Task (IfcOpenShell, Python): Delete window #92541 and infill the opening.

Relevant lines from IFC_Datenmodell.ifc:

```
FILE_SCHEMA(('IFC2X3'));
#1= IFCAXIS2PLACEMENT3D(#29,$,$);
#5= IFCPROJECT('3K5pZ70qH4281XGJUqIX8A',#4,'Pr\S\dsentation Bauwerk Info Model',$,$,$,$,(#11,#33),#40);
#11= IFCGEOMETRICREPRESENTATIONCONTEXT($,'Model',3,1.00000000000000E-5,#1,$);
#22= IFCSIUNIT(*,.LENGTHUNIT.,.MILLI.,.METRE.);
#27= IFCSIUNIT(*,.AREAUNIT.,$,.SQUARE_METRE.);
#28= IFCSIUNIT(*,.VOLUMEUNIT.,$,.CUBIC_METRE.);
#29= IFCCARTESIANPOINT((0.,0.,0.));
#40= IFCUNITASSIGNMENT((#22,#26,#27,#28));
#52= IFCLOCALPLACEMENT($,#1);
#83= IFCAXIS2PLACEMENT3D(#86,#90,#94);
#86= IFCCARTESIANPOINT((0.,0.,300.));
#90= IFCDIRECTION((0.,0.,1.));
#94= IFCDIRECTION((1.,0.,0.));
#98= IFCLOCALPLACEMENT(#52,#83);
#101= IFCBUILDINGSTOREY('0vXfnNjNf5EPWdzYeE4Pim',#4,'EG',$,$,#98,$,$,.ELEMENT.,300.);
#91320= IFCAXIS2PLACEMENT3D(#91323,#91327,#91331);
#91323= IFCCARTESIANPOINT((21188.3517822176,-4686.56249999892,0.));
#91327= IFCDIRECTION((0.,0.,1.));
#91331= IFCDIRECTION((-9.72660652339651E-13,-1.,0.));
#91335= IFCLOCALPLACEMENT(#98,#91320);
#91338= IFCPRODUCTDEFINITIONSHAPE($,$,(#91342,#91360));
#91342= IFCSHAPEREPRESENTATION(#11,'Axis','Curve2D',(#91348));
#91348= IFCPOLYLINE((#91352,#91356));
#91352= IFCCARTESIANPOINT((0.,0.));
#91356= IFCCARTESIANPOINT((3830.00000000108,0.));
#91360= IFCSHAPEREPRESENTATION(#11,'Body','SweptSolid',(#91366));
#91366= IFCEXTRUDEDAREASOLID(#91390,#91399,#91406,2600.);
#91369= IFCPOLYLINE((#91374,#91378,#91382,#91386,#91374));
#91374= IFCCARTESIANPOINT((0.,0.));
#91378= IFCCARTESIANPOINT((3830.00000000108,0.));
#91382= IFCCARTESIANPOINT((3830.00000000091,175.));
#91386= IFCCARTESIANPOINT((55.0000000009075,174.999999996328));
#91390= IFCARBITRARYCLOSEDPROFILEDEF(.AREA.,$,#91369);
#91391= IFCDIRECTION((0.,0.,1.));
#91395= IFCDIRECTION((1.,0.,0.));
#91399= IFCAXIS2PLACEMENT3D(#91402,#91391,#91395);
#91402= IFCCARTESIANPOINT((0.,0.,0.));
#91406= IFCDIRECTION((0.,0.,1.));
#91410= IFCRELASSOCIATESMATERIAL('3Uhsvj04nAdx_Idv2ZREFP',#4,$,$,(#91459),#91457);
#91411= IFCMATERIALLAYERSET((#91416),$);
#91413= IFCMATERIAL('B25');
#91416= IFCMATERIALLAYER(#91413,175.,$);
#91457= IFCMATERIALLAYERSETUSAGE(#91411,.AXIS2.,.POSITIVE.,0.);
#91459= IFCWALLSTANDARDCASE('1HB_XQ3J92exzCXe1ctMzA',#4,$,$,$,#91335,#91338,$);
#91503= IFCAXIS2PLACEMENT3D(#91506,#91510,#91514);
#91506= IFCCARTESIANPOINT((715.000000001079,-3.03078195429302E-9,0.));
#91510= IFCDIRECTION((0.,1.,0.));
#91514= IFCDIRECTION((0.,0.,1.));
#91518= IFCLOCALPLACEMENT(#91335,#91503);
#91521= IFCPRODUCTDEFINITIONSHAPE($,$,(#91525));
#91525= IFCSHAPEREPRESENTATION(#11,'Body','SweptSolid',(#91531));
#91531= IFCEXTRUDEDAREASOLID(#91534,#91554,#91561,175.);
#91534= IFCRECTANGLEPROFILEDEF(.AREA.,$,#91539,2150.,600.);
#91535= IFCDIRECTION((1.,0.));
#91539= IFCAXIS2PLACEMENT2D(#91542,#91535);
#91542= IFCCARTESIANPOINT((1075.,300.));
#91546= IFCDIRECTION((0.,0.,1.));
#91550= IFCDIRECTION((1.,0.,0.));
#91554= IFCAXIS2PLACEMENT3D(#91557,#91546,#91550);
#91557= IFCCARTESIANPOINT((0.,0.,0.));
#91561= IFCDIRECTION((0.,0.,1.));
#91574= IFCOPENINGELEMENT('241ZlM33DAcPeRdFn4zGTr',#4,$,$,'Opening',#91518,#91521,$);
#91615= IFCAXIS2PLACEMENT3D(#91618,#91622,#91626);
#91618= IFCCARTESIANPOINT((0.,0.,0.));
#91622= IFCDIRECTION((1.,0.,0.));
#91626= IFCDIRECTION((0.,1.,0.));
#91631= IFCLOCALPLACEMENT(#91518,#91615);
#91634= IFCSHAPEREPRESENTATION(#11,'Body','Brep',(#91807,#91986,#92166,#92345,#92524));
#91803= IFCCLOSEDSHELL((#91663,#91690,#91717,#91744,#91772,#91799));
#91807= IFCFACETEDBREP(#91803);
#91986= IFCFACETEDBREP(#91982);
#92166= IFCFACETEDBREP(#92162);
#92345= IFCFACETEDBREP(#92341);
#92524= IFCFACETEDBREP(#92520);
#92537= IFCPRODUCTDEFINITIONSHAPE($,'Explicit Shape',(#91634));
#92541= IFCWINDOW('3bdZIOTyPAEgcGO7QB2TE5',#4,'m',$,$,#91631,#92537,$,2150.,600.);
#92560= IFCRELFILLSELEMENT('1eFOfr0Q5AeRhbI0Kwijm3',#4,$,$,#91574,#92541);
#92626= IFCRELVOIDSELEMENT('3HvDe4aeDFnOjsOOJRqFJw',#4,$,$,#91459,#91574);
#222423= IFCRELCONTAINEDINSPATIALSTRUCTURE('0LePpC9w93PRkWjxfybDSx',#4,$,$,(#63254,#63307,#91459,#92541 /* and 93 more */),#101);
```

```python
import ifcopenshell
import ifcopenshell.api.feature
import ifcopenshell.api.root
import ifcopenshell.geom
import ifcopenshell.util.shape

model = ifcopenshell.open("IFC_Datenmodell.ifc")
settings = ifcopenshell.geom.settings()


def volume(element):
    """Net volume in cubic metres, openings subtracted."""
    shape = ifcopenshell.geom.create_shape(settings, element)
    return ifcopenshell.util.shape.get_volume(shape.geometry)


window = model.by_guid("3bdZIOTyPAEgcGO7QB2TE5")
opening = window.FillsVoids[0].RelatingOpeningElement
wall = opening.VoidsElements[0].RelatingBuildingElement
before = volume(wall)

ifcopenshell.api.root.remove_product(model, product=window)
ifcopenshell.api.feature.remove_feature(model, feature=opening)

after = volume(wall)

print(f"wall volume {before:.3f} -> {after:.3f} m3")

model.write("IFC_Datenmodell_updated.ifc")
```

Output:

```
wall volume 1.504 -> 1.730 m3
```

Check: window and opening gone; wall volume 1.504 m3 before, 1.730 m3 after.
